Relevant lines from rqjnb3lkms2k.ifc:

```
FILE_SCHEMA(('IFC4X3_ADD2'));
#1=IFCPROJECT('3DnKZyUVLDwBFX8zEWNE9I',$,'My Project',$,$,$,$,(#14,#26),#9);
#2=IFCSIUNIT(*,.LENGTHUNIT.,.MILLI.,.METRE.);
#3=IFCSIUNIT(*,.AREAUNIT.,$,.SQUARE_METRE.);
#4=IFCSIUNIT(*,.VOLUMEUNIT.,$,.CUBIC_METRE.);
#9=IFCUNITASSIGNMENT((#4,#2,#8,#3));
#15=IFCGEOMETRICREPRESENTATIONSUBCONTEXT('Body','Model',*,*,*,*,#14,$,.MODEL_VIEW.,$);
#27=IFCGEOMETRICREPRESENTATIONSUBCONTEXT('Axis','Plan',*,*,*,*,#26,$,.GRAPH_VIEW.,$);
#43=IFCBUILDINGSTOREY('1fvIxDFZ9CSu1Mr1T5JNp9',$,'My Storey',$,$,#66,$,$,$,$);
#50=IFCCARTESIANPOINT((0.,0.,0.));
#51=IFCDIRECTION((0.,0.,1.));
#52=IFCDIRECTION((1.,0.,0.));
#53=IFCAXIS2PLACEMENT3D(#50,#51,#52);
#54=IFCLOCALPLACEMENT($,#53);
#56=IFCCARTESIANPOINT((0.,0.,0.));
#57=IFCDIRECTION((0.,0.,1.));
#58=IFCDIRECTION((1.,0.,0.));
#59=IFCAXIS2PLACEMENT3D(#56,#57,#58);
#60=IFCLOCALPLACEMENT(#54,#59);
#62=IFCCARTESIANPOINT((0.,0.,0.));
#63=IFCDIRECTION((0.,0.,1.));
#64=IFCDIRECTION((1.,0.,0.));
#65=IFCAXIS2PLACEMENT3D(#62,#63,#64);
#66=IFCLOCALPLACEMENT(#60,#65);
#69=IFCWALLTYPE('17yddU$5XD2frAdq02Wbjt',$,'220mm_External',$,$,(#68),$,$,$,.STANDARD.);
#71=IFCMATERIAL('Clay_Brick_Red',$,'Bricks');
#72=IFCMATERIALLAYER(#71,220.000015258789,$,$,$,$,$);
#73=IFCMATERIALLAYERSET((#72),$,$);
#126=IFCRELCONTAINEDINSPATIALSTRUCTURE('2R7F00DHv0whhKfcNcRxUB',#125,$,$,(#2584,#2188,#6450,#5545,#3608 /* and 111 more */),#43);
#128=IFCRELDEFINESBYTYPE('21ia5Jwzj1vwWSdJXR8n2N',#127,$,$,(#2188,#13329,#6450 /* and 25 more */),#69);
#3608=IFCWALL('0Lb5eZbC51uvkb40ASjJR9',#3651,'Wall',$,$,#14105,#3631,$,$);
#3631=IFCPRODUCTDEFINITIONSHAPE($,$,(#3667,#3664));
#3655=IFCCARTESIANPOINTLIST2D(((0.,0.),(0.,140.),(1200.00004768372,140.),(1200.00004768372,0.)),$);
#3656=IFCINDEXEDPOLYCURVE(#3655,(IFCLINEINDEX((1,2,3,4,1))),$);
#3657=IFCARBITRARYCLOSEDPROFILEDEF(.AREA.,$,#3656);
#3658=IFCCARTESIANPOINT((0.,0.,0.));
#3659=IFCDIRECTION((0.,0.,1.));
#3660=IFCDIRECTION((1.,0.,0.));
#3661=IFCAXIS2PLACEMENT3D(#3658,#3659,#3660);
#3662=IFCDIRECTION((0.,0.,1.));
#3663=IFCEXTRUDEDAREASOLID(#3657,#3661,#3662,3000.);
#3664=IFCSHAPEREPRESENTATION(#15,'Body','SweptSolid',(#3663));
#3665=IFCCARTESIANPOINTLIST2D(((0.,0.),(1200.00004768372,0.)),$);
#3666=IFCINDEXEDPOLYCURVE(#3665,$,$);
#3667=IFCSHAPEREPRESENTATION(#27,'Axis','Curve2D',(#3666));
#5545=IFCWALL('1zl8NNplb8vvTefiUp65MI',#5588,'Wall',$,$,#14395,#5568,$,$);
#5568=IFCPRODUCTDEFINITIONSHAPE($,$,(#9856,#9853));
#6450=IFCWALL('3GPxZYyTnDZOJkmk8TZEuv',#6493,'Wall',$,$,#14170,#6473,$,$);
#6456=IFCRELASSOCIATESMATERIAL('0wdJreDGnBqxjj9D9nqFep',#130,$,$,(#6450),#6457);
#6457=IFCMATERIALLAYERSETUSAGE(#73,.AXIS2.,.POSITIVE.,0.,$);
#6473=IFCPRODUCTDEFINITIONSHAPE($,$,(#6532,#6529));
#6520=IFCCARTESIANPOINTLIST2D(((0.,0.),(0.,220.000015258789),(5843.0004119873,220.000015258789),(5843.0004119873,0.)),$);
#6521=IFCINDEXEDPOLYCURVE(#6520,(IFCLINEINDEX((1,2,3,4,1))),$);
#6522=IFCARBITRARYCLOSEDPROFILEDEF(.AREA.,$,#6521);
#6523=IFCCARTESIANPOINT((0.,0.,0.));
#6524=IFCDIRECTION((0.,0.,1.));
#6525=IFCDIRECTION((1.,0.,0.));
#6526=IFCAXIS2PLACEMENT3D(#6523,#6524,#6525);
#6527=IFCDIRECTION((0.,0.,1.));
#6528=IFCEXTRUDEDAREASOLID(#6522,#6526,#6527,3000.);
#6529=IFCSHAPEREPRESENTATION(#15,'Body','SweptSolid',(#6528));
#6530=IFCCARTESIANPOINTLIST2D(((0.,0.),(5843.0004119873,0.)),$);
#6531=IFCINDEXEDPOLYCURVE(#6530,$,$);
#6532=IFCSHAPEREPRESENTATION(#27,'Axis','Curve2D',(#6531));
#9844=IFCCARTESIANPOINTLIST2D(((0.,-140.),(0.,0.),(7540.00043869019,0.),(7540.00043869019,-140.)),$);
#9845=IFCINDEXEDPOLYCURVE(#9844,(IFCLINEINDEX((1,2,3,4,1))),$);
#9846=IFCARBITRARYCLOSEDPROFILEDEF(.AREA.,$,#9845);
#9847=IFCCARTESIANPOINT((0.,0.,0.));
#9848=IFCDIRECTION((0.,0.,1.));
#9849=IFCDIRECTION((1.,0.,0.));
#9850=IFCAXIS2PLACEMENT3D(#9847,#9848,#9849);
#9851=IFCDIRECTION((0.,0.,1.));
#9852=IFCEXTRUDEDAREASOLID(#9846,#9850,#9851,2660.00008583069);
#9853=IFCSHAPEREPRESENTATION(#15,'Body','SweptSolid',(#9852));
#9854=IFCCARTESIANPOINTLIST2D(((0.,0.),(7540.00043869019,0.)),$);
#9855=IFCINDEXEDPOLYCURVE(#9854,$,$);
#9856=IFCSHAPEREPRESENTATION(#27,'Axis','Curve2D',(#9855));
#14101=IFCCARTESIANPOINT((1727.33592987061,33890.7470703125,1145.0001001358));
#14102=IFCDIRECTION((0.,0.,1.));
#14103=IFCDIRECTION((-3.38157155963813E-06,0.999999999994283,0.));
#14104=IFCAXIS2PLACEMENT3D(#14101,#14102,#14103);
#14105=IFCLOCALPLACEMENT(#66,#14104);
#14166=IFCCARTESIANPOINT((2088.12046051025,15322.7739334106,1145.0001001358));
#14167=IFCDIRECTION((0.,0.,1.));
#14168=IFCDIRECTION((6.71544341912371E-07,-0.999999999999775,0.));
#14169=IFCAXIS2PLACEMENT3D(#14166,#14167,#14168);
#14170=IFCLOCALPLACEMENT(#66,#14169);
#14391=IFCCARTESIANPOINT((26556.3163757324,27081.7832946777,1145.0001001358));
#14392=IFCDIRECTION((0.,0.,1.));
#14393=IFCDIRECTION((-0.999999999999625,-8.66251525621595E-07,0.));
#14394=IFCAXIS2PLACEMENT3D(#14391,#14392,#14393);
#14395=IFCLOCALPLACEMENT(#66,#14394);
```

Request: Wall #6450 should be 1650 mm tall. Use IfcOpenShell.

```python
import ifcopenshell
import ifcopenshell.geom
import ifcopenshell.util.representation
import ifcopenshell.util.shape
import ifcopenshell.util.unit

model = ifcopenshell.open("rqjnb3lkms2k.ifc")
unit_scale = ifcopenshell.util.unit.calculate_unit_scale(model)
settings = ifcopenshell.geom.settings()


def volume(element):
    """Net volume in cubic metres, openings subtracted."""
    shape = ifcopenshell.geom.create_shape(settings, element)
    return ifcopenshell.util.shape.get_volume(shape.geometry)


wall = model.by_id(6450)
before = volume(wall)

body = ifcopenshell.util.representation.get_representation(wall, "Model", "Body")
solid = body.Items[0]
old_height = solid.Depth
solid.Depth = 1.65 / unit_scale
after = volume(wall)

print(f"height {old_height:g} -> {solid.Depth:g}, volume {before:.3f} -> {after:.3f} m3")

model.write("rqjnb3lkms2k_edited.ifc")
```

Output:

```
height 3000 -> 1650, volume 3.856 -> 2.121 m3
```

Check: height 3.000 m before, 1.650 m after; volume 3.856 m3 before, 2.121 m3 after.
